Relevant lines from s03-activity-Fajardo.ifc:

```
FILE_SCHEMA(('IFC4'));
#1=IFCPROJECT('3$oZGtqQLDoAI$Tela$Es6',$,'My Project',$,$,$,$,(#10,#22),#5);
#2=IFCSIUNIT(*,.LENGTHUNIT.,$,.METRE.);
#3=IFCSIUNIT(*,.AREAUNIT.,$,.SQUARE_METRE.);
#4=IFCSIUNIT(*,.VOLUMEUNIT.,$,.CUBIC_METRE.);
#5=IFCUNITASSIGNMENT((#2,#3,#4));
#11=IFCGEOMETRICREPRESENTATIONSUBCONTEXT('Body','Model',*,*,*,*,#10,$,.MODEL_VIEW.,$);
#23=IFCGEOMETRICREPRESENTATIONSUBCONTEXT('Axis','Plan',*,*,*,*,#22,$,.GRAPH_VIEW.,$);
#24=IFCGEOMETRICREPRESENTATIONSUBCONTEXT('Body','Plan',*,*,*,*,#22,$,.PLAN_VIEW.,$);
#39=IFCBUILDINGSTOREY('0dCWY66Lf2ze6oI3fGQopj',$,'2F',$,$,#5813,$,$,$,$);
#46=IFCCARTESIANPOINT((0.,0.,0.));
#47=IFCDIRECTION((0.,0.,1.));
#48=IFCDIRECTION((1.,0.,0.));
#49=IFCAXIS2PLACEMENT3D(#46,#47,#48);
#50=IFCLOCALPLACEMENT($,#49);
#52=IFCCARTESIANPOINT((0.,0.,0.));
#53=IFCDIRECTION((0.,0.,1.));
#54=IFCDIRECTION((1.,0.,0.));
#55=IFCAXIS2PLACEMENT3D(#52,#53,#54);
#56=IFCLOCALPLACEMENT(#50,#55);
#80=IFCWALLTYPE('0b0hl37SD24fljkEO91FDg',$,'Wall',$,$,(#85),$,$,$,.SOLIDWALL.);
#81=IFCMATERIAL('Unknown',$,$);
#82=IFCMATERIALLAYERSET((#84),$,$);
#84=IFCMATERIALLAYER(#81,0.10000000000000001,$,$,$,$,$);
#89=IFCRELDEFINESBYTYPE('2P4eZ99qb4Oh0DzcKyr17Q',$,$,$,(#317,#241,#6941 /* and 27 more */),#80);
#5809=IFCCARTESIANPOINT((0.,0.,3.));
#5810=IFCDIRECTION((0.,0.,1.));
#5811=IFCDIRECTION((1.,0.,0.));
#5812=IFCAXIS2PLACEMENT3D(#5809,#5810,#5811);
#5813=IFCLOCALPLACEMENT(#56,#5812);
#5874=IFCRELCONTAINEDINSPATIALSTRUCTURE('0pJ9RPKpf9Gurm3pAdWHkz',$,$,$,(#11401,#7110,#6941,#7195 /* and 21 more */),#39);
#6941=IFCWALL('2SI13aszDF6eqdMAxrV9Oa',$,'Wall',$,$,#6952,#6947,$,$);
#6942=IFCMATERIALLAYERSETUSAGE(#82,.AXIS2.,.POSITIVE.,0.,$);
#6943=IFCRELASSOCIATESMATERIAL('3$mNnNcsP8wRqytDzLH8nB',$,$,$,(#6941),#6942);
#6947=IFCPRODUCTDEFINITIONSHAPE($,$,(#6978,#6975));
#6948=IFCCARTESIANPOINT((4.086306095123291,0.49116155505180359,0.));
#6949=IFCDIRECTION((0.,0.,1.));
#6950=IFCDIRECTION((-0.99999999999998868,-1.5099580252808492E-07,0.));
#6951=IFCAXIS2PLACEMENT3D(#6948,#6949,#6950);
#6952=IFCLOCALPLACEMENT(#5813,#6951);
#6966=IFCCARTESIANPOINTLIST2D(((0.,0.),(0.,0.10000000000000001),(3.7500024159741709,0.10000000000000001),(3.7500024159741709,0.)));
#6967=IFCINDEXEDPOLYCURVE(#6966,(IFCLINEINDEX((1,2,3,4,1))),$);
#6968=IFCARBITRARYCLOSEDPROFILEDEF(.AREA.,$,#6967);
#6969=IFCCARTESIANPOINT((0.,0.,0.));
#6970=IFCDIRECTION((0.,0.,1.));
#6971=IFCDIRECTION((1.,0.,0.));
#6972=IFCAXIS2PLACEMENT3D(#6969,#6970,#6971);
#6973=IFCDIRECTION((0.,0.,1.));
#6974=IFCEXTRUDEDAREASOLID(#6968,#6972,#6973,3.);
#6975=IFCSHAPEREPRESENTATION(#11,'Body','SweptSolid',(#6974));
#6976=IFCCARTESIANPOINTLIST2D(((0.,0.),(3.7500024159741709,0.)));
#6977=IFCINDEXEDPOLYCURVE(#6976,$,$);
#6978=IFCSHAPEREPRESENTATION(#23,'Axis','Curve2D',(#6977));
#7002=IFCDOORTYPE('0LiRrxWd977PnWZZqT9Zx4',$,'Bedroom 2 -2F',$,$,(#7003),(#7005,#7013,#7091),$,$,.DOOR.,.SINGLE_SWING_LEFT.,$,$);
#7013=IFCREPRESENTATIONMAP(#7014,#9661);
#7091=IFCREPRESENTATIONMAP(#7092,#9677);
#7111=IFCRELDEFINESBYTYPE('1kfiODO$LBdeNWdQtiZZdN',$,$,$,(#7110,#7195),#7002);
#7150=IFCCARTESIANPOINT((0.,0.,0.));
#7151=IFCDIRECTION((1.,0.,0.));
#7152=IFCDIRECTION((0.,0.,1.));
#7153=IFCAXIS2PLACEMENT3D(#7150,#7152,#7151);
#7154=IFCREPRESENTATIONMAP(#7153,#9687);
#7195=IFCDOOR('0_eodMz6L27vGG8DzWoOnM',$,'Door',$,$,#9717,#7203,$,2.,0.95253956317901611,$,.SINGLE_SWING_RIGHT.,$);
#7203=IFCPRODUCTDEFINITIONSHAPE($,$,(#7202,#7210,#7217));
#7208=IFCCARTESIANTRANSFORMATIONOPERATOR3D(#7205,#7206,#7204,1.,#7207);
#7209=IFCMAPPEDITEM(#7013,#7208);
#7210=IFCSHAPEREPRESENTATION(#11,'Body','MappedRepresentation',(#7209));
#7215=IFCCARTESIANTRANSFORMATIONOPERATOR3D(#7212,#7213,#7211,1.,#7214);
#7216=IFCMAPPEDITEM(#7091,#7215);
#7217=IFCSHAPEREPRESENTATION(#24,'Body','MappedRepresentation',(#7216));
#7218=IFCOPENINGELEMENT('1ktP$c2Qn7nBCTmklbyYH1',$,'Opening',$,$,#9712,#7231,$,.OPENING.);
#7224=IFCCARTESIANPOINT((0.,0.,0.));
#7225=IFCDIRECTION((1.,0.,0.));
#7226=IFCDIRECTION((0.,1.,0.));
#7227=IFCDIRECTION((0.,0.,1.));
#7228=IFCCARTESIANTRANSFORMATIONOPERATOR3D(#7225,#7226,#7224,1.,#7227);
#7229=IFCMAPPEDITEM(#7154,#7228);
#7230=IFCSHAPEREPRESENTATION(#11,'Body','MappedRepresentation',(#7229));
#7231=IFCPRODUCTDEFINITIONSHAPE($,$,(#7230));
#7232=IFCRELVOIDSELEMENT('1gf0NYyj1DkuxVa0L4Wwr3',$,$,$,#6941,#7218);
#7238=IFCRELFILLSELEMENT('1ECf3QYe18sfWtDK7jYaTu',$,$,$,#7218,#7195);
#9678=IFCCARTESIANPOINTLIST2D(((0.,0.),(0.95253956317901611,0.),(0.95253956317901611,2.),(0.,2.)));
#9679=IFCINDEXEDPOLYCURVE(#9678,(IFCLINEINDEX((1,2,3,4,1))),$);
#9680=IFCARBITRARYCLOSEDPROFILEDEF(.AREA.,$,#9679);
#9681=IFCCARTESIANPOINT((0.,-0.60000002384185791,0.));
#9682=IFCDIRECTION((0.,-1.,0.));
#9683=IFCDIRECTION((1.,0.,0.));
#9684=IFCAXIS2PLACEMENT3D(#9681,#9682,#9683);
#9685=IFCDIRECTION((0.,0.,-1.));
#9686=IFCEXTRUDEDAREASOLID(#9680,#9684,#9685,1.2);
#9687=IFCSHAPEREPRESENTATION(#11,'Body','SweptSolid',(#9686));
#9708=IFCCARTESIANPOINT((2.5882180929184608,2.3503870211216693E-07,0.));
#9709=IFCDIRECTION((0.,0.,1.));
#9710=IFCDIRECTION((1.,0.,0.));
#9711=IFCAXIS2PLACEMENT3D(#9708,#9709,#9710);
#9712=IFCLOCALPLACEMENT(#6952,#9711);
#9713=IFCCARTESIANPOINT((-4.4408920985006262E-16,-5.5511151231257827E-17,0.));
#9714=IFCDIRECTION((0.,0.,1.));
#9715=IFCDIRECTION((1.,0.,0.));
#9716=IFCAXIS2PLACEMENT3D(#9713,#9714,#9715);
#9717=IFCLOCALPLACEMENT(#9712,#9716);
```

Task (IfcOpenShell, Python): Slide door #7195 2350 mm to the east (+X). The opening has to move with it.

```python
import ifcopenshell
import ifcopenshell.api.geometry
import ifcopenshell.util.placement

model = ifcopenshell.open("s03-activity-Fajardo.ifc")

door = model.by_guid("0_eodMz6L27vGG8DzWoOnM")
opening = door.FillsVoids[0].RelatingOpeningElement
wall = opening.VoidsElements[0].RelatingBuildingElement

wall_matrix = ifcopenshell.util.placement.get_local_placement(wall.ObjectPlacement)
shift = wall_matrix[:3, 0] * -2.35
before = ifcopenshell.util.placement.get_local_placement(door.ObjectPlacement)[:3, 3].copy()

# The door is placed relative to its opening, so it follows when the opening moves.
matrix = ifcopenshell.util.placement.get_local_placement(opening.ObjectPlacement)
matrix[:3, 3] += shift
ifcopenshell.api.geometry.edit_object_placement(
    model, product=opening, matrix=matrix, is_si=False, should_transform_children=True
)

after = ifcopenshell.util.placement.get_local_placement(door.ObjectPlacement)[:3, 3]
print("door moved by", (after - before).round(3) + 0.0)

model.write("s03-activity-Fajardo_updated.ifc")
```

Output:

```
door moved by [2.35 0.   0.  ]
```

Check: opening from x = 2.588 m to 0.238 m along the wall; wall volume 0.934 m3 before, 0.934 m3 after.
